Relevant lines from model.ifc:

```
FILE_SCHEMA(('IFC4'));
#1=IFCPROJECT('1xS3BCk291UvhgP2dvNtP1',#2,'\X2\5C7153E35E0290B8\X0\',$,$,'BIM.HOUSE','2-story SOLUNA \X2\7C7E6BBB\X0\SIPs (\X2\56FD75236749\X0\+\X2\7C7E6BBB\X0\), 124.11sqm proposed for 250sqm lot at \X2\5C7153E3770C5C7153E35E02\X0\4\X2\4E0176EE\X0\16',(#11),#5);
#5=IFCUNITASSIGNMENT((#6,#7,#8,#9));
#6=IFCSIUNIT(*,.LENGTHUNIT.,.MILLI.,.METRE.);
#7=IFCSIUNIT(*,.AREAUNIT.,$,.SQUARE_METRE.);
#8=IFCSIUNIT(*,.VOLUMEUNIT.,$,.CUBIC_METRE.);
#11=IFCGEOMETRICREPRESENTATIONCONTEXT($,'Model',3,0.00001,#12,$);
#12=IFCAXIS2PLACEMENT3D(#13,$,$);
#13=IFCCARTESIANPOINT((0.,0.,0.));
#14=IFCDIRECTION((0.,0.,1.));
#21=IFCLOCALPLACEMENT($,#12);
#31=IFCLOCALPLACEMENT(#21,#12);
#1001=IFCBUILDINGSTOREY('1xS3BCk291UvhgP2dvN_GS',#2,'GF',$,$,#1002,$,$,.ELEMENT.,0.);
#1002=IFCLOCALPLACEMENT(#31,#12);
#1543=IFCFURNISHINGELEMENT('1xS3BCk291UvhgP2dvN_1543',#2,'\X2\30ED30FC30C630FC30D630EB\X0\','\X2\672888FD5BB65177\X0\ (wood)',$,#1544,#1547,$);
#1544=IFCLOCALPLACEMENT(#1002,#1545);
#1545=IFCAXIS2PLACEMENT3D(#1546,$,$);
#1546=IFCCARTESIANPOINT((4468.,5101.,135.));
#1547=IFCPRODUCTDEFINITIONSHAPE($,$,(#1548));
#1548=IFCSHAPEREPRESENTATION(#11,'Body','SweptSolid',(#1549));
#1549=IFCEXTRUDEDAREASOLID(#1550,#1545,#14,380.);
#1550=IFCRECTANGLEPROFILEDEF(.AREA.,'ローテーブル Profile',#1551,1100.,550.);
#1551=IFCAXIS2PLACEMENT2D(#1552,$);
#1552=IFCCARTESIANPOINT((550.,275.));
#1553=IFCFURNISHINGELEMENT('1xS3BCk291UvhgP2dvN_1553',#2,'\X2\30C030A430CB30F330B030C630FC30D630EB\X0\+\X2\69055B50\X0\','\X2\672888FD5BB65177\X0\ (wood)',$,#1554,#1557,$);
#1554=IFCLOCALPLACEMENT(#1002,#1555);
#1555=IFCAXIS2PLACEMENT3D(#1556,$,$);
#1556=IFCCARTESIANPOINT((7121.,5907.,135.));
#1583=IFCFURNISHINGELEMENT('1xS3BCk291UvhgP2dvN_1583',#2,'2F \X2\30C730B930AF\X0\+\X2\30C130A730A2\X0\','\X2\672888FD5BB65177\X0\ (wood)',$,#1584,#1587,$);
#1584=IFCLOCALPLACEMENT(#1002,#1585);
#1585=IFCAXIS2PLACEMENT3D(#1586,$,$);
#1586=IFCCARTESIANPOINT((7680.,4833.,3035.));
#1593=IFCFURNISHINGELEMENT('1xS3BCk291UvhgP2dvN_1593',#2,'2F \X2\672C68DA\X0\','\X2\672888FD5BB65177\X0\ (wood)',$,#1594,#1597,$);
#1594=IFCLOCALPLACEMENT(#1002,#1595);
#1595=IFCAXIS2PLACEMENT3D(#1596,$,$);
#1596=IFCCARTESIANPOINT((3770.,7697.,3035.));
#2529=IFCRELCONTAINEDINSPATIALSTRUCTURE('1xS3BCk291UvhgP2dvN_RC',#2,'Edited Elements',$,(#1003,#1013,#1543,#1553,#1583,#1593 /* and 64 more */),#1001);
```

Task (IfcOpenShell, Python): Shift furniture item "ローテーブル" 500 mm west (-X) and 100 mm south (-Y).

```python
import ifcopenshell
import ifcopenshell.api.geometry
import ifcopenshell.util.placement
import ifcopenshell.util.unit

model = ifcopenshell.open("model.ifc")
unit_scale = ifcopenshell.util.unit.calculate_unit_scale(model)

item = model.by_id(1543)
matrix = ifcopenshell.util.placement.get_local_placement(item.ObjectPlacement)
matrix[0, 3] -= 0.5 / unit_scale
matrix[1, 3] -= 0.1 / unit_scale
ifcopenshell.api.geometry.edit_object_placement(model, product=item, matrix=matrix, is_si=False)

print(ifcopenshell.util.placement.get_local_placement(item.ObjectPlacement).round(3) + 0.0)

model.write("model_updated.ifc")
```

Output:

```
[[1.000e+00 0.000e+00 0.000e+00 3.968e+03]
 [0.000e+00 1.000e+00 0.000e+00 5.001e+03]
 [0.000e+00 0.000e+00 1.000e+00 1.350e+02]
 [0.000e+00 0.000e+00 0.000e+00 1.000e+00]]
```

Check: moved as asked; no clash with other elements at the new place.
